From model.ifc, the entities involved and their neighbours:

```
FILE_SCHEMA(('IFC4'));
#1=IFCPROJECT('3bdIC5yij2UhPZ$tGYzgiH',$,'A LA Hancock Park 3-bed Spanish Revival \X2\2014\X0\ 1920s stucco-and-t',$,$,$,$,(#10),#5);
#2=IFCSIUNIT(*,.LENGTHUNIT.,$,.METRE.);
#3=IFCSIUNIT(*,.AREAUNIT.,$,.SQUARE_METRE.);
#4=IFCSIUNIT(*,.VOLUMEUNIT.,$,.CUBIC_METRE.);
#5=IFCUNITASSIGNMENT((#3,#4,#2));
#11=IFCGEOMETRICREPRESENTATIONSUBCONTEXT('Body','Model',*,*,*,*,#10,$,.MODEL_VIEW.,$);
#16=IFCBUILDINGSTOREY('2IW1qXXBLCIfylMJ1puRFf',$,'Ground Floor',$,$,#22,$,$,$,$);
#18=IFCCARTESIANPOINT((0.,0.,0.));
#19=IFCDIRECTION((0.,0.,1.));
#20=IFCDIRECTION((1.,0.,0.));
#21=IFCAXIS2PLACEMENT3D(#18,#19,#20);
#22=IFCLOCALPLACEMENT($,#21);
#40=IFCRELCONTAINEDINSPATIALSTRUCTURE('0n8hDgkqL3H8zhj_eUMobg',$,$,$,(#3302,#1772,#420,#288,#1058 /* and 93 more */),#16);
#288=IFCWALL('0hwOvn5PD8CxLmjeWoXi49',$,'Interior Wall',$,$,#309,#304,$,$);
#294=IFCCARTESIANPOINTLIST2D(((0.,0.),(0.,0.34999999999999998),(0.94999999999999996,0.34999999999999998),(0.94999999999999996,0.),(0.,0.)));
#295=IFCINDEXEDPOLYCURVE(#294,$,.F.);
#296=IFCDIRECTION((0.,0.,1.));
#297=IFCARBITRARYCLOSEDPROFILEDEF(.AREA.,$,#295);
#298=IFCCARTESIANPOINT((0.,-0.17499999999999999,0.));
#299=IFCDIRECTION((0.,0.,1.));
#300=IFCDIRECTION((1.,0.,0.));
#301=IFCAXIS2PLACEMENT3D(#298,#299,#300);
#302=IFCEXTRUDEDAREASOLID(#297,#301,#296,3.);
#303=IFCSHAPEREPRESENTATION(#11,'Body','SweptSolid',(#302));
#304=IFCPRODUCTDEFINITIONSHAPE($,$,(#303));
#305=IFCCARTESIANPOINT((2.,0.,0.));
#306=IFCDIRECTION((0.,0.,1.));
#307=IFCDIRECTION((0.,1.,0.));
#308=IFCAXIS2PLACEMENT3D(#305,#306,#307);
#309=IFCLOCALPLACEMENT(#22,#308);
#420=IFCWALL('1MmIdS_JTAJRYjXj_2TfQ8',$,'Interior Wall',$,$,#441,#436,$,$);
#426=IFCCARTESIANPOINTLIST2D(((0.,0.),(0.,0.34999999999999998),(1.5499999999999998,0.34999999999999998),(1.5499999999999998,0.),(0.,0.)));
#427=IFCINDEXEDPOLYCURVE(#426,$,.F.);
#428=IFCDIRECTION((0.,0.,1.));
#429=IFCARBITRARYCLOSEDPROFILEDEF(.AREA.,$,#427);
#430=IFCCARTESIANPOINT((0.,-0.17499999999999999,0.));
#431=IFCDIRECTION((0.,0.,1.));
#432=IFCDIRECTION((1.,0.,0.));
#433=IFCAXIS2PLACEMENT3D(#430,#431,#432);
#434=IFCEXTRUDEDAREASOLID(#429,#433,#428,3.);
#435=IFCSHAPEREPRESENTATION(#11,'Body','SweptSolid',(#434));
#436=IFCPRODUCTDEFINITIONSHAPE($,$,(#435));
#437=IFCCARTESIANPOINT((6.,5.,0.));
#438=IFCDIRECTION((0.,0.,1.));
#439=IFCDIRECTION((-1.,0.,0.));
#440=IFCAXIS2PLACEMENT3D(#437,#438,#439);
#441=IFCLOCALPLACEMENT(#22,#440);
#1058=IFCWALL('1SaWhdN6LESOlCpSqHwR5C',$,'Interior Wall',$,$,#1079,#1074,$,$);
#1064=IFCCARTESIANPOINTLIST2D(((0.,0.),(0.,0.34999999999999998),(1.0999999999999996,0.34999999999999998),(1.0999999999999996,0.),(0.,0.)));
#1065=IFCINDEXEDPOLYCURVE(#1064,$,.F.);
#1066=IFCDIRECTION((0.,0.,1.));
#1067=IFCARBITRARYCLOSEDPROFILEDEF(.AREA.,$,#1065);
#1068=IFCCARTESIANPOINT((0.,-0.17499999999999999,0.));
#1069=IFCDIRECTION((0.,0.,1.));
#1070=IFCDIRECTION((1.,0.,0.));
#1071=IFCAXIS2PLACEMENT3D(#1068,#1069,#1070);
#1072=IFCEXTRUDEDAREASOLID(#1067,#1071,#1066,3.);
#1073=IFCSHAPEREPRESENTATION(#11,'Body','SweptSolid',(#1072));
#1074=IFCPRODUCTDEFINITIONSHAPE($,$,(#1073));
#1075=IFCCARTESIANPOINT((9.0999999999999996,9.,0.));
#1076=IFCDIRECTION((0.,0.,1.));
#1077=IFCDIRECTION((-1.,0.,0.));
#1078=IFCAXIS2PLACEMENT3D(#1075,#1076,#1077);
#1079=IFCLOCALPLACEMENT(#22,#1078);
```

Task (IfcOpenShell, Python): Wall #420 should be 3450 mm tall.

```python
import ifcopenshell
import ifcopenshell.geom
import ifcopenshell.util.representation
import ifcopenshell.util.shape
import ifcopenshell.util.unit

model = ifcopenshell.open("model.ifc")
unit_scale = ifcopenshell.util.unit.calculate_unit_scale(model)
settings = ifcopenshell.geom.settings()


def volume(element):
    """Net volume in cubic metres, openings subtracted."""
    shape = ifcopenshell.geom.create_shape(settings, element)
    return ifcopenshell.util.shape.get_volume(shape.geometry)


wall = model.by_id(420)
before = volume(wall)

body = ifcopenshell.util.representation.get_representation(wall, "Model", "Body")
solid = body.Items[0]
old_height = solid.Depth
solid.Depth = 3.45 / unit_scale
after = volume(wall)

print(f"height {old_height:g} -> {solid.Depth:g}, volume {before:.3f} -> {after:.3f} m3")

model.write("model-out.ifc")
```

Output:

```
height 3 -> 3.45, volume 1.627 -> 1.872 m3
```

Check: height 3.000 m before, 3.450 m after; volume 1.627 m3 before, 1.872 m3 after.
